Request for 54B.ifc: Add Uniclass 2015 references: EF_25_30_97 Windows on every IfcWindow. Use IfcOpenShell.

First a look at what the model holds.

```python
import ifcopenshell

model = ifcopenshell.open("54B.ifc")
print(model.schema)
print("classifications:", [c.Name for c in model.by_type("IfcClassification")])
for ifc_class in ("IfcDoor", "IfcRoof", "IfcStair", "IfcWall", "IfcWindow"):
    print(ifc_class, len(model.by_type(ifc_class)))
```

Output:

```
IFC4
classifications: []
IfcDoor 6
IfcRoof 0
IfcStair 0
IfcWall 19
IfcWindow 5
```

```python
import ifcopenshell
import ifcopenshell.api.classification

model = ifcopenshell.open("54B.ifc")

system = ifcopenshell.api.classification.add_classification(model, classification="Uniclass 2015")

codes = {
    "IfcWindow": ("EF_25_30_97", "Windows"),
}
for ifc_class, (code, name) in codes.items():
    products = model.by_type(ifc_class)
    ifcopenshell.api.classification.add_reference(
        model, products=products, classification=system, identification=code, name=name
    )
    print(code, len(products))

model.write("54B_edited.ifc")
```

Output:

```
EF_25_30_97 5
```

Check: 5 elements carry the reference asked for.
